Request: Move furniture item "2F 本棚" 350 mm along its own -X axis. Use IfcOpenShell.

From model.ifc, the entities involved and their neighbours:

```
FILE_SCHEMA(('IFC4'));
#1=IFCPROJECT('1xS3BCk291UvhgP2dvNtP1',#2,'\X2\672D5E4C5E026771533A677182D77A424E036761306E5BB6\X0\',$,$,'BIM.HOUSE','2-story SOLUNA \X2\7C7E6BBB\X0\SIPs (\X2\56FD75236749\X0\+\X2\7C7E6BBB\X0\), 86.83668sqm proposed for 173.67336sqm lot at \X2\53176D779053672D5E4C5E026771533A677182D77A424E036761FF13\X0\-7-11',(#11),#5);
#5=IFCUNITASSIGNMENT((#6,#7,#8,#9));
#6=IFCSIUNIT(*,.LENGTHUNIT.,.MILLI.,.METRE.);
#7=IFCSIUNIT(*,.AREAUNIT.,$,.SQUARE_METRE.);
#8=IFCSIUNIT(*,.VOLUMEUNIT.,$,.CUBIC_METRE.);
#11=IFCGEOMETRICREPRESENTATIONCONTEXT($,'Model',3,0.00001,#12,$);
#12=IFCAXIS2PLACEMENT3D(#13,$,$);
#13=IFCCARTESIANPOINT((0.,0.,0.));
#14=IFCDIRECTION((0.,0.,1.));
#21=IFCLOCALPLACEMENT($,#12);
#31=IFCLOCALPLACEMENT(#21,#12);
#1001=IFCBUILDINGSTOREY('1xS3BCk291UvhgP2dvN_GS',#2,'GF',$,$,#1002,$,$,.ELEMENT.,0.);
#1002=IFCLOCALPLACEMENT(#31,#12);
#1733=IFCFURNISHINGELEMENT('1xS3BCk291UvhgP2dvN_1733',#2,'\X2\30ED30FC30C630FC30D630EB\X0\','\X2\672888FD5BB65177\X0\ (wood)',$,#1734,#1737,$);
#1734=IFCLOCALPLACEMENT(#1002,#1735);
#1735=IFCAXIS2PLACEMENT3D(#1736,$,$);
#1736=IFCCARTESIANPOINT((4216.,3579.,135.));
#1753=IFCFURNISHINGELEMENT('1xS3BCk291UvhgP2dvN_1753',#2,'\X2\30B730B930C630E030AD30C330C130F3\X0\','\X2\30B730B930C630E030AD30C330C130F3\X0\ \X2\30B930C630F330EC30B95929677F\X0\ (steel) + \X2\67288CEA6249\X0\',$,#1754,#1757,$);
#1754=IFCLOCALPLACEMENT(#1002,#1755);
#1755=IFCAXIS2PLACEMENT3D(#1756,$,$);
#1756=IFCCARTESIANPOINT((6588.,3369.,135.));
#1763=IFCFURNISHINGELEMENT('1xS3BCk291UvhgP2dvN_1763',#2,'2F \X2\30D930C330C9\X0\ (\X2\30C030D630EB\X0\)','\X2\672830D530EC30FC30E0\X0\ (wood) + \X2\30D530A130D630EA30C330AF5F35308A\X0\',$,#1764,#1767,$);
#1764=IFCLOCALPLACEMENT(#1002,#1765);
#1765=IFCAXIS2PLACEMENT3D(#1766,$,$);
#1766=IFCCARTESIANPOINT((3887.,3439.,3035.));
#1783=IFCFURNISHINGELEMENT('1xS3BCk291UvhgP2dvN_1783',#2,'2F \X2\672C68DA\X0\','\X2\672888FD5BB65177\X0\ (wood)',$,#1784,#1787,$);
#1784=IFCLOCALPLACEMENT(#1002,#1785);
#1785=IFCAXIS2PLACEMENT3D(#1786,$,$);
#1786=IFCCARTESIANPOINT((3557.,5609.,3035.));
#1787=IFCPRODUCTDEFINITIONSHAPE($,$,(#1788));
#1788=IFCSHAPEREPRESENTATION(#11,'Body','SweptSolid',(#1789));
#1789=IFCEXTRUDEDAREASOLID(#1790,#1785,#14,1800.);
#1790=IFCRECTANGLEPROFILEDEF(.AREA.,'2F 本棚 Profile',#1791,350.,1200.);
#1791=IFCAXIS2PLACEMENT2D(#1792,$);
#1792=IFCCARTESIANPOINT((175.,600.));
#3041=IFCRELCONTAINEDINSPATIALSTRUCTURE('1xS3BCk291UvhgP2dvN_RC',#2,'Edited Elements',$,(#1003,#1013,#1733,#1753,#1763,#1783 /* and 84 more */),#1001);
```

```python
import ifcopenshell
import ifcopenshell.api.geometry
import ifcopenshell.util.placement
import ifcopenshell.util.unit

model = ifcopenshell.open("model.ifc")
unit_scale = ifcopenshell.util.unit.calculate_unit_scale(model)

item = model.by_guid("1xS3BCk291UvhgP2dvN_1783")
matrix = ifcopenshell.util.placement.get_local_placement(item.ObjectPlacement)
matrix[:3, 3] -= matrix[:3, 0] * 0.35 / unit_scale
ifcopenshell.api.geometry.edit_object_placement(model, product=item, matrix=matrix, is_si=False)

print(ifcopenshell.util.placement.get_local_placement(item.ObjectPlacement).round(3) + 0.0)

model.write("model_edited.ifc")
```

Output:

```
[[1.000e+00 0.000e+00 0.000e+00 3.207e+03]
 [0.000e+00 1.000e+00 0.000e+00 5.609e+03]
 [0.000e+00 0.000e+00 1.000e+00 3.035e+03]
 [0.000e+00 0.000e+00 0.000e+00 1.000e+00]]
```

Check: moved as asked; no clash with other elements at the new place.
